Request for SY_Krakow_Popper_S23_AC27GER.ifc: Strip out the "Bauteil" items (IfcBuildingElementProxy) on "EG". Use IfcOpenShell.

First a look at what the model holds.

```python
import ifcopenshell
import ifcopenshell.util.element

model = ifcopenshell.open("SY_Krakow_Popper_S23_AC27GER.ifc")
print(model.schema)
storey = next(s for s in model.by_type("IfcBuildingStorey") if s.Name == "EG")
proxies = [e for e in ifcopenshell.util.element.get_decomposition(storey) if e.is_a("IfcBuildingElementProxy")]
seen = {}
for e in proxies:
    element_type = ifcopenshell.util.element.get_type(e)
    name = element_type.Name if element_type not in (None, e) else None
    seen[name] = seen.get(name, 0) + 1
for name, count in sorted(seen.items(), key=str):
    print(count, "x", name)
```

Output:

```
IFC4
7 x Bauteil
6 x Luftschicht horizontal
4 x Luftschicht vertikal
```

```python
import ifcopenshell
import ifcopenshell.api.root
import ifcopenshell.util.element

model = ifcopenshell.open("SY_Krakow_Popper_S23_AC27GER.ifc")

storey = next(s for s in model.by_type("IfcBuildingStorey") if s.Name == "EG")
proxies = [e for e in ifcopenshell.util.element.get_decomposition(storey) if e.is_a("IfcBuildingElementProxy")]
targets = [e for e in proxies if (t := ifcopenshell.util.element.get_type(e)) not in (None, e) and t.Name == "Bauteil"]

for e in targets:
    ifcopenshell.api.root.remove_product(model, product=e)
print(len(targets), "removed")

model.write("SY_Krakow_Popper_S23_AC27GER_updated.ifc")
```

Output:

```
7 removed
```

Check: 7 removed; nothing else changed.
